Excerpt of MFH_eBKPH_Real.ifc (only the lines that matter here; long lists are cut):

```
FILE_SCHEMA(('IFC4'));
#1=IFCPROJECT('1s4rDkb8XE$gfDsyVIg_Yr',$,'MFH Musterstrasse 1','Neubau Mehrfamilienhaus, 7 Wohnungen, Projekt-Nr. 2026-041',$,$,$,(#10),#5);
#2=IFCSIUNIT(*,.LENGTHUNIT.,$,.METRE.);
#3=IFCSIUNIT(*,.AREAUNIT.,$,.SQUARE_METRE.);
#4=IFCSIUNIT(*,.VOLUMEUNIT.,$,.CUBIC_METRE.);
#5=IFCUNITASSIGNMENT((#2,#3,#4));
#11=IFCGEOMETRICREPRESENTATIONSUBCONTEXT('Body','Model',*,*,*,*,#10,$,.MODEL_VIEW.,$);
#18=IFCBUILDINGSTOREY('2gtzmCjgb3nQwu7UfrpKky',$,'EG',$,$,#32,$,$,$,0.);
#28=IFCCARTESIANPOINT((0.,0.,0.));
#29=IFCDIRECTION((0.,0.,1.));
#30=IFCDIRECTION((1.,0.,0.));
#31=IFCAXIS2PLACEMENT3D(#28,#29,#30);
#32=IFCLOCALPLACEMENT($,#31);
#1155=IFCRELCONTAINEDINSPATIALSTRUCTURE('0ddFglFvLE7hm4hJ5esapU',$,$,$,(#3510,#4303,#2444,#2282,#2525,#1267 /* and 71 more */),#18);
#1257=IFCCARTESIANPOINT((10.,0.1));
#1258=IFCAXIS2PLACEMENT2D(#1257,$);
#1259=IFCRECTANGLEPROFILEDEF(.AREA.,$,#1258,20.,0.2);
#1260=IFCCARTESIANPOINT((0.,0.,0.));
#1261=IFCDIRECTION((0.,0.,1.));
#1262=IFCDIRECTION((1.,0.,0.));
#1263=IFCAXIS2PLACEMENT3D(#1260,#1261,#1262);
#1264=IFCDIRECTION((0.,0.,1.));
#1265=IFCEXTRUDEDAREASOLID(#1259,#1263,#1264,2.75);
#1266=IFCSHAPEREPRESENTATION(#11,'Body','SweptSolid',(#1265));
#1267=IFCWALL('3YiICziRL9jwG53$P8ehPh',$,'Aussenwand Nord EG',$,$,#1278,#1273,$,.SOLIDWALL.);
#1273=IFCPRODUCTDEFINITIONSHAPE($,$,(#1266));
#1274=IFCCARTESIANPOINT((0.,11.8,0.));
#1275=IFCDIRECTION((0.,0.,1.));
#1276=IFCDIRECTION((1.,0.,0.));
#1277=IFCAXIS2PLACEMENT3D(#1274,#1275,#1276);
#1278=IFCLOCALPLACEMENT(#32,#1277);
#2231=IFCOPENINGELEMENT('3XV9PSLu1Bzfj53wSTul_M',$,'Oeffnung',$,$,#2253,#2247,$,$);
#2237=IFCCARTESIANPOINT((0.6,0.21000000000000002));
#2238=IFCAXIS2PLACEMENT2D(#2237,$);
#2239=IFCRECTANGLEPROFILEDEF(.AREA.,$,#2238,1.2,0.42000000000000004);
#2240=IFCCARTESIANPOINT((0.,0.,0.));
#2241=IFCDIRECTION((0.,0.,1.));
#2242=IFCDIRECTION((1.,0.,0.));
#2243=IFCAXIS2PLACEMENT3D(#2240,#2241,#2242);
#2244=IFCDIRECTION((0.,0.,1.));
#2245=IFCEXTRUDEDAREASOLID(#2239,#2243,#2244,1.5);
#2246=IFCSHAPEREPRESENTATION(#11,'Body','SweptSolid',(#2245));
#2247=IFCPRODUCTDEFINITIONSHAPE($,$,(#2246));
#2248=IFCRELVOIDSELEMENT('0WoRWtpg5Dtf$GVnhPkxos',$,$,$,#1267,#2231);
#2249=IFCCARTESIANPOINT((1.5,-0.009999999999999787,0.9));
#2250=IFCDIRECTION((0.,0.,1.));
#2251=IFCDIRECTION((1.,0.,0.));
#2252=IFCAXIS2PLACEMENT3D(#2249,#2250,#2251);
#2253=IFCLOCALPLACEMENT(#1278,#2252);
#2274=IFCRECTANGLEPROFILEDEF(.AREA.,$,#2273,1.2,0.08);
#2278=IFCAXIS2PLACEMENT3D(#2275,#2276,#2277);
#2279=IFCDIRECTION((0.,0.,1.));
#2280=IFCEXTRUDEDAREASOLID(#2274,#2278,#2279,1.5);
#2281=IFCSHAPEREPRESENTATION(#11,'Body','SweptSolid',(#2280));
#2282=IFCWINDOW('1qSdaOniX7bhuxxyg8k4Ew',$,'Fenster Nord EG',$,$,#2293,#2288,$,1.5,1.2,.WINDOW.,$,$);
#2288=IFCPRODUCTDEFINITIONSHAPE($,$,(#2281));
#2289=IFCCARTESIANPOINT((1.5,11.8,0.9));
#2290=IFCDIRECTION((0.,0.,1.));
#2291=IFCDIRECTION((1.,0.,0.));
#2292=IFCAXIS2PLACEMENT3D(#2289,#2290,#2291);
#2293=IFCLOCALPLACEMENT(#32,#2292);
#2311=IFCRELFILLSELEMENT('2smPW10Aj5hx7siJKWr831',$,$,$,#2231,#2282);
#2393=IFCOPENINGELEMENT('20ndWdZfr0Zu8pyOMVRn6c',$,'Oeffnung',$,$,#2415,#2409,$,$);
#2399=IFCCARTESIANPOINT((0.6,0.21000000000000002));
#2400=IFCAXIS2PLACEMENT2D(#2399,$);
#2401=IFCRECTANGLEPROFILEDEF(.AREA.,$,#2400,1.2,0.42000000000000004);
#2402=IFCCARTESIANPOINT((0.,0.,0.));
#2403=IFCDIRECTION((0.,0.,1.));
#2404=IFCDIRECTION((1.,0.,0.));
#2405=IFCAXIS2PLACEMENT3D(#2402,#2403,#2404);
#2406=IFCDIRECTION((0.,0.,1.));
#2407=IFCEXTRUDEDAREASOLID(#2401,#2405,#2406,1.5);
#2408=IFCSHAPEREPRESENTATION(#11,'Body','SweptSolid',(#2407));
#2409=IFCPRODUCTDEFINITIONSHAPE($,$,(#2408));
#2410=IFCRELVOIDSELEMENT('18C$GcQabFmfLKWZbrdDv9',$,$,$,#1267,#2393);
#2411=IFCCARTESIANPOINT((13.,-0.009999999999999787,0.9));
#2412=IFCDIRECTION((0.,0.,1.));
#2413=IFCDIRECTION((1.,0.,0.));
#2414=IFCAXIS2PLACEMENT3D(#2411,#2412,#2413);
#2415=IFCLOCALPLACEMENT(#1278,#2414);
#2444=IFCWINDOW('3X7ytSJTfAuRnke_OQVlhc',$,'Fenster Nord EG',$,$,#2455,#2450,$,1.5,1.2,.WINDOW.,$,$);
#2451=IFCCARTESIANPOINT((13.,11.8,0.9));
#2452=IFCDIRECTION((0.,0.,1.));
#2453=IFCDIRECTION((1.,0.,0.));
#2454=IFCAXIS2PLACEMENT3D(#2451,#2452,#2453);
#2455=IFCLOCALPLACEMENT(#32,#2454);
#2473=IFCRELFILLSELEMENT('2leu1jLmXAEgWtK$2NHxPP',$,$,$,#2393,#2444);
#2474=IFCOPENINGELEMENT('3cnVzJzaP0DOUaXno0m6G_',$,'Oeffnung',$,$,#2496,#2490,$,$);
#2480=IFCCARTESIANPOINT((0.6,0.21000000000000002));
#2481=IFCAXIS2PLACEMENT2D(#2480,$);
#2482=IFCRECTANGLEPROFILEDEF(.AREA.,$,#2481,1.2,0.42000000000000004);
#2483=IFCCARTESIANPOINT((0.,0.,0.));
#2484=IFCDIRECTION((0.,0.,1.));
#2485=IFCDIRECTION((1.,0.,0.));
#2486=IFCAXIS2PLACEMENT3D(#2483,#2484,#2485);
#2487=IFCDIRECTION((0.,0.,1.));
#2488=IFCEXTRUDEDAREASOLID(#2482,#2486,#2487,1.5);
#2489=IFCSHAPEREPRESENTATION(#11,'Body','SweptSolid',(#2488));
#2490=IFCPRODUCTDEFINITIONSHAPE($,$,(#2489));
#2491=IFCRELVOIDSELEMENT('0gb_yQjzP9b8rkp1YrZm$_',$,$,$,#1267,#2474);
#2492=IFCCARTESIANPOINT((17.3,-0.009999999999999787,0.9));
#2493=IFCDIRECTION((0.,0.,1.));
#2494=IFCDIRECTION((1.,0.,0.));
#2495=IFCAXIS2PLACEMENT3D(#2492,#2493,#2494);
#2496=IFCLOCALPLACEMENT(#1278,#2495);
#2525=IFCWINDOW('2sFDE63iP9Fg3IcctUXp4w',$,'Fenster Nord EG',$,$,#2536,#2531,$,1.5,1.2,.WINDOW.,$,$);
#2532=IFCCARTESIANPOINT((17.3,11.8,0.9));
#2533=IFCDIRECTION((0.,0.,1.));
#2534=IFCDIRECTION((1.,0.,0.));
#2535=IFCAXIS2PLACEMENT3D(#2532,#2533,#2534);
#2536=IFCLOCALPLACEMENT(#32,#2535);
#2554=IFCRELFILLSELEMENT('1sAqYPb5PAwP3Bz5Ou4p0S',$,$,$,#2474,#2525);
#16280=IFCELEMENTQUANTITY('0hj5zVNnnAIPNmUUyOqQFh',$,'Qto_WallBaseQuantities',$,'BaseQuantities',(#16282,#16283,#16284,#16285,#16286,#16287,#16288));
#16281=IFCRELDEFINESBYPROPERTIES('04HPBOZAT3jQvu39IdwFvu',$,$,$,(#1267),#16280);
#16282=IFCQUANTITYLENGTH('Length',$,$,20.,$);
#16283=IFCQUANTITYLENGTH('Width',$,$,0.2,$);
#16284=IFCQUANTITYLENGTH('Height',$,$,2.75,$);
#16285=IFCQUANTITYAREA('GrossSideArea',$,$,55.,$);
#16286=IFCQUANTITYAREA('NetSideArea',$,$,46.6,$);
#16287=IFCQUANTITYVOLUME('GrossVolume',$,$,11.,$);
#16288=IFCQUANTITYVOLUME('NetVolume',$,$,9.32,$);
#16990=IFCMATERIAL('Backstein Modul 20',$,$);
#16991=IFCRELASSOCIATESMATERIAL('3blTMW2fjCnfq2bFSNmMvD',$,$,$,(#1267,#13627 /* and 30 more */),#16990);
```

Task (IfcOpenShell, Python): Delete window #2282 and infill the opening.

```python
import ifcopenshell
import ifcopenshell.api.feature
import ifcopenshell.api.pset
import ifcopenshell.api.root
import ifcopenshell.geom
import ifcopenshell.util.element
import ifcopenshell.util.shape
import ifcopenshell.util.unit

model = ifcopenshell.open("MFH_eBKPH_Real.ifc")
area_scale = ifcopenshell.util.unit.calculate_unit_scale(model, "AREAUNIT")
volume_scale = ifcopenshell.util.unit.calculate_unit_scale(model, "VOLUMEUNIT")
settings = ifcopenshell.geom.settings()


def volume(element):
    """Net volume in cubic metres, openings subtracted."""
    shape = ifcopenshell.geom.create_shape(settings, element)
    return ifcopenshell.util.shape.get_volume(shape.geometry)


window = model.by_id(2282)
opening = window.FillsVoids[0].RelatingOpeningElement
wall = opening.VoidsElements[0].RelatingBuildingElement
before = volume(wall)

ifcopenshell.api.root.remove_product(model, product=window)
ifcopenshell.api.feature.remove_feature(model, feature=opening)

after = volume(wall)
thickness = 0.2  # wall thickness in metres

# Update the wall's stored quantities.
qto = model.by_id(ifcopenshell.util.element.get_pset(wall, "Qto_WallBaseQuantities", should_inherit=False)["id"])
ifcopenshell.api.pset.edit_qto(model, qto=qto, properties={
    "NetSideArea": after / thickness / area_scale,
    "NetVolume": after / volume_scale,
})

print(f"wall volume {before:.3f} -> {after:.3f} m3")

model.write("MFH_eBKPH_Real_rev.ifc")
```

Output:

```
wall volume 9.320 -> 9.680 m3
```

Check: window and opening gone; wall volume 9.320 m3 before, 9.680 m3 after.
